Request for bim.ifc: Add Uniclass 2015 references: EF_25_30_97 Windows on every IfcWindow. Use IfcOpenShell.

First a look at what the model holds.

```python
import ifcopenshell

model = ifcopenshell.open("bim.ifc")
print(model.schema)
print("classifications:", [c.Name for c in model.by_type("IfcClassification")])
for ifc_class in ("IfcDoor", "IfcRoof", "IfcStair", "IfcWall", "IfcWindow"):
    print(ifc_class, len(model.by_type(ifc_class)))
```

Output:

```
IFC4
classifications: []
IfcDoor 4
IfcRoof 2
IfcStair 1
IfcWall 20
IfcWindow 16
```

```python
import ifcopenshell
import ifcopenshell.api.classification

model = ifcopenshell.open("bim.ifc")

system = ifcopenshell.api.classification.add_classification(model, classification="Uniclass 2015")

codes = {
    "IfcWindow": ("EF_25_30_97", "Windows"),
}
for ifc_class, (code, name) in codes.items():
    products = model.by_type(ifc_class)
    ifcopenshell.api.classification.add_reference(
        model, products=products, classification=system, identification=code, name=name
    )
    print(code, len(products))

model.write("bim_updated.ifc")
```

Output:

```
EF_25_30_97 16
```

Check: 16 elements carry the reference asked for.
